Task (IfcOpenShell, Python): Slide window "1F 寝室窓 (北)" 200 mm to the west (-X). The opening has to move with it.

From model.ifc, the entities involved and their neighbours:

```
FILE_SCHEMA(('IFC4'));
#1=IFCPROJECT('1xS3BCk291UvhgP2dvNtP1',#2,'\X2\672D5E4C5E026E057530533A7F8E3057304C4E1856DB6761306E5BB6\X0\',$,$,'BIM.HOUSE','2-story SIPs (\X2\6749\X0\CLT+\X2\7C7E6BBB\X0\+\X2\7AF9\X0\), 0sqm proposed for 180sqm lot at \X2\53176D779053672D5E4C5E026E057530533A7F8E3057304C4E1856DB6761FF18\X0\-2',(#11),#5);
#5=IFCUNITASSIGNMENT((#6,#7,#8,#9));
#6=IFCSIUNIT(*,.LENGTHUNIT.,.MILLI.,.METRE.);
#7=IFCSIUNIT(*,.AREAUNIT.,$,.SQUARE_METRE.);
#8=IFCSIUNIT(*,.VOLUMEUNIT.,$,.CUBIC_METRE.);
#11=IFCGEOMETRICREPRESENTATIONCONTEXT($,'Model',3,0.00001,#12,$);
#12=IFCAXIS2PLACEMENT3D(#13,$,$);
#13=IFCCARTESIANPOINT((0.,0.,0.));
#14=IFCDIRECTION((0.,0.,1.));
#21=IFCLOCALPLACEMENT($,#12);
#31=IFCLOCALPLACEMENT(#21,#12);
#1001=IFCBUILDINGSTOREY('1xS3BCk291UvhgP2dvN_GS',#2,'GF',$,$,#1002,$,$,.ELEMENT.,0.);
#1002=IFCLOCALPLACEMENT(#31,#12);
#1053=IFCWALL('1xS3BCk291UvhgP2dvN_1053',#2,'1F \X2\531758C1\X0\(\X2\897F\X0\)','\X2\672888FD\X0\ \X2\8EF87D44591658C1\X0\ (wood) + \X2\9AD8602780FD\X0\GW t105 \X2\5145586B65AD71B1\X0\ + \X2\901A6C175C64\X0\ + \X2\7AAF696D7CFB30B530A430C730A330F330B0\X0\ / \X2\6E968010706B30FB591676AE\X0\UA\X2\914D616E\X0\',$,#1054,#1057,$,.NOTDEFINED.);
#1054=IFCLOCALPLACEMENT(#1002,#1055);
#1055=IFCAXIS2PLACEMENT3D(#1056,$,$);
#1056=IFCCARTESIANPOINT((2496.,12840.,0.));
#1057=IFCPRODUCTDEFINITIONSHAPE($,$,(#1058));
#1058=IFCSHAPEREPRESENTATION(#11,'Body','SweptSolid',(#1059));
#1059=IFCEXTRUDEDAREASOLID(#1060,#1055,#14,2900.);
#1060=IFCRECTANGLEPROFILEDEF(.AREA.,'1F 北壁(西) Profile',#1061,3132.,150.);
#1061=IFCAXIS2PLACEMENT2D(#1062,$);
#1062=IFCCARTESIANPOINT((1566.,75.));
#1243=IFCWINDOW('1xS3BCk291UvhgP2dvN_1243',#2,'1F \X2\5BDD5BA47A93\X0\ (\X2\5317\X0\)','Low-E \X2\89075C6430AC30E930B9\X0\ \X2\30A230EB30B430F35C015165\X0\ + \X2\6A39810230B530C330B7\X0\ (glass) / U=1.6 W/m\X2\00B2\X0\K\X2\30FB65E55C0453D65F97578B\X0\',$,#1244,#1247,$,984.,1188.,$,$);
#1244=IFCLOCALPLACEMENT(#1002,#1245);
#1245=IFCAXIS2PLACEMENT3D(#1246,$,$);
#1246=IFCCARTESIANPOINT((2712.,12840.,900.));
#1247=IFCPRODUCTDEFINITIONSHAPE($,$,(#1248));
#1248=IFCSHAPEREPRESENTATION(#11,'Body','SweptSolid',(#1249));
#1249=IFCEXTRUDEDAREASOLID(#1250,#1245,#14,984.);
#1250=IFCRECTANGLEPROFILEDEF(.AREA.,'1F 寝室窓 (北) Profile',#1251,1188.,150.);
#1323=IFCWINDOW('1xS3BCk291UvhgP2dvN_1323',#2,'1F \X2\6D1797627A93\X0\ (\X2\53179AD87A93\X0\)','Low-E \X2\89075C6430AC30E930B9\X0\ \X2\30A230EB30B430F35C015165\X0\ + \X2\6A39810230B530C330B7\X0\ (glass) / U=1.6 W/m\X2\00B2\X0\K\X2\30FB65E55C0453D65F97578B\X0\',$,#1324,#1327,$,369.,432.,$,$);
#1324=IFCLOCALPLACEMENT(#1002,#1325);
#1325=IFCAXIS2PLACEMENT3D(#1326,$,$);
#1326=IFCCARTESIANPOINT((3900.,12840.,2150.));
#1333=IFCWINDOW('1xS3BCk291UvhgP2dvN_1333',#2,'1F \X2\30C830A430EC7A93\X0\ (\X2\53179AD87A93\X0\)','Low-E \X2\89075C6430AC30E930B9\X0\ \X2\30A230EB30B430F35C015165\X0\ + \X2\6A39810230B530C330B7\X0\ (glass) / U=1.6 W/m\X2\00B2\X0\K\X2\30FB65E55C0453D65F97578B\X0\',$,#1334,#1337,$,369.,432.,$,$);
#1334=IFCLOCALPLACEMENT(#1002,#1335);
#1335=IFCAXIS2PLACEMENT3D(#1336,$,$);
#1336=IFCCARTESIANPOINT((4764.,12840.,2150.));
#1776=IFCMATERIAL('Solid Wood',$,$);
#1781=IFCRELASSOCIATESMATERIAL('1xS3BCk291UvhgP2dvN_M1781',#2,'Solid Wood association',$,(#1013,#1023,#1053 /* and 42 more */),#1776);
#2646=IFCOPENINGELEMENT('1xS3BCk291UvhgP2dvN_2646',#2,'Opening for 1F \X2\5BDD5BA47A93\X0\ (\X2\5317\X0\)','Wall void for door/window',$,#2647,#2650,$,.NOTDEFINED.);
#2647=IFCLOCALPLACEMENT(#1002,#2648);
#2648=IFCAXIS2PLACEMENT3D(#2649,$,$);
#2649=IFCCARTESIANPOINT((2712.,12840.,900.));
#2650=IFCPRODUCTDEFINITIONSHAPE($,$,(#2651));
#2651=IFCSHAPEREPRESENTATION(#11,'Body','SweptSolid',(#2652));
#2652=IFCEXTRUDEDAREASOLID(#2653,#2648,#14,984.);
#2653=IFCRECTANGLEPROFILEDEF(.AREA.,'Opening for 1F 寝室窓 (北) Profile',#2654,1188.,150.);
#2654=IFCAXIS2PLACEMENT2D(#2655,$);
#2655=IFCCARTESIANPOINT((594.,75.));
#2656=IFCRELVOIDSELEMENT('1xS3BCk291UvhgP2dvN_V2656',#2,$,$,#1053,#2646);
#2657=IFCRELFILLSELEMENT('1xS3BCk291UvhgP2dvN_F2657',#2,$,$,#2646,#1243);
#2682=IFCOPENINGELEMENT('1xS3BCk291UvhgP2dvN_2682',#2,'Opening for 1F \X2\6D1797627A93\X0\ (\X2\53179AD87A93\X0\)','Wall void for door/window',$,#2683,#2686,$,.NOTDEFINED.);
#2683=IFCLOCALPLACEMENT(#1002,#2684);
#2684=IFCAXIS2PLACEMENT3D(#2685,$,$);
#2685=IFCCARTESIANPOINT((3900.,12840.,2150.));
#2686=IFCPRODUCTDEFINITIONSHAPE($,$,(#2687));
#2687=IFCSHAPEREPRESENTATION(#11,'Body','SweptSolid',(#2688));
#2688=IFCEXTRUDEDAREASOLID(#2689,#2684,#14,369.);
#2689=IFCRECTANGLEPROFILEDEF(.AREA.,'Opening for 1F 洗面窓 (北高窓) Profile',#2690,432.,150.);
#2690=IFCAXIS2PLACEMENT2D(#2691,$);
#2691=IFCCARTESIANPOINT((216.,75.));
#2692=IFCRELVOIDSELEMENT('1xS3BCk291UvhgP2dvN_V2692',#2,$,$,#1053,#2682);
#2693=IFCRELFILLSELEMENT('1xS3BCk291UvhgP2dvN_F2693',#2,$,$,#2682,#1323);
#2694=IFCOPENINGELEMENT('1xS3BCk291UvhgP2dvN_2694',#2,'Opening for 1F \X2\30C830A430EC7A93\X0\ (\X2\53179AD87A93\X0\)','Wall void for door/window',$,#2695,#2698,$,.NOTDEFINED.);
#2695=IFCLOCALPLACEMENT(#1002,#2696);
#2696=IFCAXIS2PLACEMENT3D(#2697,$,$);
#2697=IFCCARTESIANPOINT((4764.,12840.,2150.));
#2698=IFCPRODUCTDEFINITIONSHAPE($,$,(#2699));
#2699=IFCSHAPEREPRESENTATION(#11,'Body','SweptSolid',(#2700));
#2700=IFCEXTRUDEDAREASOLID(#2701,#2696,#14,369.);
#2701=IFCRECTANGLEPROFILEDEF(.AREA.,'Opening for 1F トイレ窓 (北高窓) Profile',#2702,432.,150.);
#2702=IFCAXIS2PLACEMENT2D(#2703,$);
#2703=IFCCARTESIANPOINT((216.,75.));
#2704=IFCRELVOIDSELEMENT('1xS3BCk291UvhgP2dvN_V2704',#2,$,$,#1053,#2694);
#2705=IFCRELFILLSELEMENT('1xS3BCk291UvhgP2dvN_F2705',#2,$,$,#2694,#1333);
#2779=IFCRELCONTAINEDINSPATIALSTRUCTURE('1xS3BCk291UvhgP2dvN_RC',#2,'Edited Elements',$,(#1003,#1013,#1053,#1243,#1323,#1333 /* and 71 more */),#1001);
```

```python
import ifcopenshell
import ifcopenshell.api.geometry
import ifcopenshell.util.placement
import ifcopenshell.util.unit

model = ifcopenshell.open("model.ifc")
unit_scale = ifcopenshell.util.unit.calculate_unit_scale(model)

window = model.by_guid("1xS3BCk291UvhgP2dvN_1243")
opening = window.FillsVoids[0].RelatingOpeningElement
wall = opening.VoidsElements[0].RelatingBuildingElement

wall_matrix = ifcopenshell.util.placement.get_local_placement(wall.ObjectPlacement)
shift = wall_matrix[:3, 0] * -0.2 / unit_scale
before = ifcopenshell.util.placement.get_local_placement(window.ObjectPlacement)[:3, 3].copy()

# The window is not placed relative to its opening, so move both.
for product in (opening, window):
    matrix = ifcopenshell.util.placement.get_local_placement(product.ObjectPlacement)
    matrix[:3, 3] += shift
    ifcopenshell.api.geometry.edit_object_placement(model, product=product, matrix=matrix, is_si=False)

after = ifcopenshell.util.placement.get_local_placement(window.ObjectPlacement)[:3, 3]
print("window moved by", (after - before).round(3) + 0.0)

model.write("model_edited.ifc")
```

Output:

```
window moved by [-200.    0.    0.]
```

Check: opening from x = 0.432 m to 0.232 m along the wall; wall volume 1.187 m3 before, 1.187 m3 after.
